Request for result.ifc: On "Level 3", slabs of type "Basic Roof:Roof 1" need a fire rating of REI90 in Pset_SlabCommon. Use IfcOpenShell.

First a look at what the model holds.

```python
import ifcopenshell
import ifcopenshell.util.element

model = ifcopenshell.open("result.ifc")
print(model.schema)
storey = next(s for s in model.by_type("IfcBuildingStorey") if s.Name == "Level 3")
slabs = [e for e in ifcopenshell.util.element.get_decomposition(storey) if e.is_a("IfcSlab")]
seen = {}
for e in slabs:
    element_type = ifcopenshell.util.element.get_type(e)
    key = (element_type.Name if element_type != e and element_type else None, ifcopenshell.util.element.get_pset(e, "Pset_SlabCommon", "FireRating"))
    seen[key] = seen.get(key, 0) + 1
for (name, value), count in sorted(seen.items(), key=str):
    print(count, "x", name, "|", value)
```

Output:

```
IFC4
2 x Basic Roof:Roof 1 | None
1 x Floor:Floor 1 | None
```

```python
import ifcopenshell
import ifcopenshell.api.pset
import ifcopenshell.util.element

model = ifcopenshell.open("result.ifc")

storey = next(s for s in model.by_type("IfcBuildingStorey") if s.Name == "Level 3")
slabs = [e for e in ifcopenshell.util.element.get_decomposition(storey) if e.is_a("IfcSlab")]

count = 0
for e in slabs:
    element_type = ifcopenshell.util.element.get_type(e)
    if element_type in (None, e) or element_type.Name != "Basic Roof:Roof 1":
        continue
    # add_pset returns the element's existing set when there is one.
    pset = ifcopenshell.api.pset.add_pset(model, product=e, name="Pset_SlabCommon")
    ifcopenshell.api.pset.edit_pset(model, pset=pset, properties={"FireRating": "REI90"})
    count += 1

print(count, "slabs updated")

model.write("result_rev.ifc")
```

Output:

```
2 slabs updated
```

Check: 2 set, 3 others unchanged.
